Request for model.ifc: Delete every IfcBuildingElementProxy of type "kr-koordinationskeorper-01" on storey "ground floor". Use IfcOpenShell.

First a look at what the model holds.

```python
import ifcopenshell
import ifcopenshell.util.element

model = ifcopenshell.open("model.ifc")
print(model.schema)
storey = next(s for s in model.by_type("IfcBuildingStorey") if s.Name == "ground floor")
proxies = [e for e in ifcopenshell.util.element.get_decomposition(storey) if e.is_a("IfcBuildingElementProxy")]
seen = {}
for e in proxies:
    element_type = ifcopenshell.util.element.get_type(e)
    name = element_type.Name if element_type not in (None, e) else None
    seen[name] = seen.get(name, 0) + 1
for name, count in sorted(seen.items(), key=str):
    print(count, "x", name)
```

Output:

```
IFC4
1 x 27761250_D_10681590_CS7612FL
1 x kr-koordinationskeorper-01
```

```python
import ifcopenshell
import ifcopenshell.api.root
import ifcopenshell.util.element

model = ifcopenshell.open("model.ifc")

storey = next(s for s in model.by_type("IfcBuildingStorey") if s.Name == "ground floor")
proxies = [e for e in ifcopenshell.util.element.get_decomposition(storey) if e.is_a("IfcBuildingElementProxy")]
targets = [e for e in proxies if (t := ifcopenshell.util.element.get_type(e)) not in (None, e) and t.Name == "kr-koordinationskeorper-01"]

for e in targets:
    ifcopenshell.api.root.remove_product(model, product=e)
print(len(targets), "removed")

model.write("model_updated.ifc")
```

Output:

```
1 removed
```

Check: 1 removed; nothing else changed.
